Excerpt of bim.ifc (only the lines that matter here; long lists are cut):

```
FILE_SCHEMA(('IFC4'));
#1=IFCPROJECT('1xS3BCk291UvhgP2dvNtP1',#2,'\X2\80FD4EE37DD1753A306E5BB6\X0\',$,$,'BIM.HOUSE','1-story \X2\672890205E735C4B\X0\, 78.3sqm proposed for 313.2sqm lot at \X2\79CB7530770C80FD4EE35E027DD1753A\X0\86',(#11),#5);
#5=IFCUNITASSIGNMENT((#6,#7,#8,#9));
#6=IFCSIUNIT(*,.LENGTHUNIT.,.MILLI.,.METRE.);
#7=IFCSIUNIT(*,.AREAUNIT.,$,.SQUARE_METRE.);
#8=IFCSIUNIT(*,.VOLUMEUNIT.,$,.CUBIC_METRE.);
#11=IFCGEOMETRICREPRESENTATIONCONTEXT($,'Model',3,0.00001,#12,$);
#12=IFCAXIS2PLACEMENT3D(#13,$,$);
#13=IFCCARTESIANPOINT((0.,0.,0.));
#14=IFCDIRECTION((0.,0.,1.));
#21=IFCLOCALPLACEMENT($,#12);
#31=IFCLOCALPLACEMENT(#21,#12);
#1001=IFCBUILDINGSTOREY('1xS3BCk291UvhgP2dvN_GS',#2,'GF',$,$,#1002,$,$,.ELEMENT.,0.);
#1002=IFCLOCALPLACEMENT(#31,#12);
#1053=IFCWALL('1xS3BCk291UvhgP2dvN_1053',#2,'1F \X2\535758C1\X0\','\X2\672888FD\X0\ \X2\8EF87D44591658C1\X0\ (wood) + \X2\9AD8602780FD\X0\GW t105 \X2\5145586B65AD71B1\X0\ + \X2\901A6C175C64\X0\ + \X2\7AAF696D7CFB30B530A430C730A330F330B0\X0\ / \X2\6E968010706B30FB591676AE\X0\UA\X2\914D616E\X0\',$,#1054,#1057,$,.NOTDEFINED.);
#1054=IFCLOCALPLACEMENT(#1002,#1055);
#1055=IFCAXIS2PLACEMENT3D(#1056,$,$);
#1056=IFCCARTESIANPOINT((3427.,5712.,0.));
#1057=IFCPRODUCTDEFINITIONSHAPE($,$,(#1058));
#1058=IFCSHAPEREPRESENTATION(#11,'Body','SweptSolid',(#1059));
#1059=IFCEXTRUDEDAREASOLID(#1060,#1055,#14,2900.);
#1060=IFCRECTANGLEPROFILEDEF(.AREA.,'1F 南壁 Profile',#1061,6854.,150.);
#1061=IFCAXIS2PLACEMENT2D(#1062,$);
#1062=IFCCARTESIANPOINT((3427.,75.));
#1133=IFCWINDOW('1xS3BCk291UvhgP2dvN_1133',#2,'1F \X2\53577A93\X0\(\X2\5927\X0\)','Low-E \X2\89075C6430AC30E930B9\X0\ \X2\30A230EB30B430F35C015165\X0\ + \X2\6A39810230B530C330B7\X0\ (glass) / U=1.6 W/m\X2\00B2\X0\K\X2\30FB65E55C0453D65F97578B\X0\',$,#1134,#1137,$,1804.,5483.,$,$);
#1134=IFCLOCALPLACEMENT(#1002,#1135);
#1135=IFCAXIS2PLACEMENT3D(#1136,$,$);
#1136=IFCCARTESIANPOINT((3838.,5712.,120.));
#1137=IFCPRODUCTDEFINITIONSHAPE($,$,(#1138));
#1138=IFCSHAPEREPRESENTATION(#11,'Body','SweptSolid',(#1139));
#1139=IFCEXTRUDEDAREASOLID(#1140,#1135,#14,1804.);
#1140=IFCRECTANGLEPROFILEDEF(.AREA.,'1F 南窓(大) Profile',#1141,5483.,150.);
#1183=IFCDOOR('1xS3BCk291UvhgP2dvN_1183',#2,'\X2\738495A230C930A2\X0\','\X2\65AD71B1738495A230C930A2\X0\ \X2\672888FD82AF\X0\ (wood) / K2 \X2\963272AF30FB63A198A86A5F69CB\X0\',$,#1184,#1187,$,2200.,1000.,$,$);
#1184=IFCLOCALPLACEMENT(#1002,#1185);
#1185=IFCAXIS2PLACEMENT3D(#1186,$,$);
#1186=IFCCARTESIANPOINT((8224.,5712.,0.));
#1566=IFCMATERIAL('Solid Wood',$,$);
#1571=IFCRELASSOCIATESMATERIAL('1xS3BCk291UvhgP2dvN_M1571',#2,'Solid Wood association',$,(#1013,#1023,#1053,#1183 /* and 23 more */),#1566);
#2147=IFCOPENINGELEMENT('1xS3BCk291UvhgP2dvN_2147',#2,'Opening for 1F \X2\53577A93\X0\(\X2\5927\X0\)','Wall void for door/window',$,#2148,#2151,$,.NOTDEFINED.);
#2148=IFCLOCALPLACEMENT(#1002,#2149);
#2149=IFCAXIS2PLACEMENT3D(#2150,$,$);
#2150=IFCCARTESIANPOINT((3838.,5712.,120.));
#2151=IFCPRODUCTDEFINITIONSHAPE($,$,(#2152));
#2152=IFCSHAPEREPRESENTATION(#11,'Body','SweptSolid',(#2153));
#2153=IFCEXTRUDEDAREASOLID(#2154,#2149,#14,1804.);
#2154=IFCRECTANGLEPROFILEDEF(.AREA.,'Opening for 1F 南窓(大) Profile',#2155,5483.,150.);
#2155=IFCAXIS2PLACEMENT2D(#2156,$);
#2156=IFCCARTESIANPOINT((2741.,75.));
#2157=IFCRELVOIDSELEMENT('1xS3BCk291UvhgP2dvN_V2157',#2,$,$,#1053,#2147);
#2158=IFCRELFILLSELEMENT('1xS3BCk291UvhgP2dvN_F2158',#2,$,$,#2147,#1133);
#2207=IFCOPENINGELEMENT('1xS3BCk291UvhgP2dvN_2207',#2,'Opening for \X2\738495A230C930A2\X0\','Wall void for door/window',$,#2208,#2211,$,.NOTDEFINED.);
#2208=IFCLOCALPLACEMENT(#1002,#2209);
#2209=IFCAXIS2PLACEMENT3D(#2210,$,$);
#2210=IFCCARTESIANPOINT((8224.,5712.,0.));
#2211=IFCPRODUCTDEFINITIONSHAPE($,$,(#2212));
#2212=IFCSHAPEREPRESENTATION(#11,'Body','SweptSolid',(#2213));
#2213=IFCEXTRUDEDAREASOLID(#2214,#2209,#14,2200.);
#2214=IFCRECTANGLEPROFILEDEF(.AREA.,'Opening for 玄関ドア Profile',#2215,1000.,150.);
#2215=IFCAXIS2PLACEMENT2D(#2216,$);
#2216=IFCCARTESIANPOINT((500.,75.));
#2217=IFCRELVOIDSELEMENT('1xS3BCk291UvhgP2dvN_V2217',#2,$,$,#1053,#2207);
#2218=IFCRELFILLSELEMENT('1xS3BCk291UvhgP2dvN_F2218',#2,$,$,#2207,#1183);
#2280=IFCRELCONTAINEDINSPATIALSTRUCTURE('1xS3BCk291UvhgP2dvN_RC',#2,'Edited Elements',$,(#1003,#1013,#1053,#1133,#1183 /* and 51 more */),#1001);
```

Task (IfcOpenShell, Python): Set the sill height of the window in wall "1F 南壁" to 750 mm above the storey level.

```python
import numpy as np
import ifcopenshell
import ifcopenshell.api.geometry
import ifcopenshell.geom
import ifcopenshell.util.element
import ifcopenshell.util.placement
import ifcopenshell.util.shape
import ifcopenshell.util.unit

model = ifcopenshell.open("bim.ifc")
unit_scale = ifcopenshell.util.unit.calculate_unit_scale(model)

window = model.by_guid("1xS3BCk291UvhgP2dvN_1133")
opening = window.FillsVoids[0].RelatingOpeningElement
storey = ifcopenshell.util.element.get_container(window, ifc_class="IfcBuildingStorey")
level = ifcopenshell.util.placement.get_local_placement(storey.ObjectPlacement)[2, 3]

# The opening's origin need not be at the sill, so measure its lowest point.
shape = ifcopenshell.geom.create_shape(ifcopenshell.geom.settings(), opening)
bottom = ifcopenshell.util.shape.get_shape_bottom_elevation(shape, shape.geometry) / unit_scale
dz = level + 0.75 / unit_scale - bottom

shift = np.array([0.0, 0.0, dz])
# The window is not placed relative to its opening, so move both.
for product in (opening, window):
    matrix = ifcopenshell.util.placement.get_local_placement(product.ObjectPlacement)
    matrix[:3, 3] += shift
    ifcopenshell.api.geometry.edit_object_placement(model, product=product, matrix=matrix, is_si=False)

print(f"moved by {dz * unit_scale:+.3f} m")

model.write("bim_edited.ifc")
```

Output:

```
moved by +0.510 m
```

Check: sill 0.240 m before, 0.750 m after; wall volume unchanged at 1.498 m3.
